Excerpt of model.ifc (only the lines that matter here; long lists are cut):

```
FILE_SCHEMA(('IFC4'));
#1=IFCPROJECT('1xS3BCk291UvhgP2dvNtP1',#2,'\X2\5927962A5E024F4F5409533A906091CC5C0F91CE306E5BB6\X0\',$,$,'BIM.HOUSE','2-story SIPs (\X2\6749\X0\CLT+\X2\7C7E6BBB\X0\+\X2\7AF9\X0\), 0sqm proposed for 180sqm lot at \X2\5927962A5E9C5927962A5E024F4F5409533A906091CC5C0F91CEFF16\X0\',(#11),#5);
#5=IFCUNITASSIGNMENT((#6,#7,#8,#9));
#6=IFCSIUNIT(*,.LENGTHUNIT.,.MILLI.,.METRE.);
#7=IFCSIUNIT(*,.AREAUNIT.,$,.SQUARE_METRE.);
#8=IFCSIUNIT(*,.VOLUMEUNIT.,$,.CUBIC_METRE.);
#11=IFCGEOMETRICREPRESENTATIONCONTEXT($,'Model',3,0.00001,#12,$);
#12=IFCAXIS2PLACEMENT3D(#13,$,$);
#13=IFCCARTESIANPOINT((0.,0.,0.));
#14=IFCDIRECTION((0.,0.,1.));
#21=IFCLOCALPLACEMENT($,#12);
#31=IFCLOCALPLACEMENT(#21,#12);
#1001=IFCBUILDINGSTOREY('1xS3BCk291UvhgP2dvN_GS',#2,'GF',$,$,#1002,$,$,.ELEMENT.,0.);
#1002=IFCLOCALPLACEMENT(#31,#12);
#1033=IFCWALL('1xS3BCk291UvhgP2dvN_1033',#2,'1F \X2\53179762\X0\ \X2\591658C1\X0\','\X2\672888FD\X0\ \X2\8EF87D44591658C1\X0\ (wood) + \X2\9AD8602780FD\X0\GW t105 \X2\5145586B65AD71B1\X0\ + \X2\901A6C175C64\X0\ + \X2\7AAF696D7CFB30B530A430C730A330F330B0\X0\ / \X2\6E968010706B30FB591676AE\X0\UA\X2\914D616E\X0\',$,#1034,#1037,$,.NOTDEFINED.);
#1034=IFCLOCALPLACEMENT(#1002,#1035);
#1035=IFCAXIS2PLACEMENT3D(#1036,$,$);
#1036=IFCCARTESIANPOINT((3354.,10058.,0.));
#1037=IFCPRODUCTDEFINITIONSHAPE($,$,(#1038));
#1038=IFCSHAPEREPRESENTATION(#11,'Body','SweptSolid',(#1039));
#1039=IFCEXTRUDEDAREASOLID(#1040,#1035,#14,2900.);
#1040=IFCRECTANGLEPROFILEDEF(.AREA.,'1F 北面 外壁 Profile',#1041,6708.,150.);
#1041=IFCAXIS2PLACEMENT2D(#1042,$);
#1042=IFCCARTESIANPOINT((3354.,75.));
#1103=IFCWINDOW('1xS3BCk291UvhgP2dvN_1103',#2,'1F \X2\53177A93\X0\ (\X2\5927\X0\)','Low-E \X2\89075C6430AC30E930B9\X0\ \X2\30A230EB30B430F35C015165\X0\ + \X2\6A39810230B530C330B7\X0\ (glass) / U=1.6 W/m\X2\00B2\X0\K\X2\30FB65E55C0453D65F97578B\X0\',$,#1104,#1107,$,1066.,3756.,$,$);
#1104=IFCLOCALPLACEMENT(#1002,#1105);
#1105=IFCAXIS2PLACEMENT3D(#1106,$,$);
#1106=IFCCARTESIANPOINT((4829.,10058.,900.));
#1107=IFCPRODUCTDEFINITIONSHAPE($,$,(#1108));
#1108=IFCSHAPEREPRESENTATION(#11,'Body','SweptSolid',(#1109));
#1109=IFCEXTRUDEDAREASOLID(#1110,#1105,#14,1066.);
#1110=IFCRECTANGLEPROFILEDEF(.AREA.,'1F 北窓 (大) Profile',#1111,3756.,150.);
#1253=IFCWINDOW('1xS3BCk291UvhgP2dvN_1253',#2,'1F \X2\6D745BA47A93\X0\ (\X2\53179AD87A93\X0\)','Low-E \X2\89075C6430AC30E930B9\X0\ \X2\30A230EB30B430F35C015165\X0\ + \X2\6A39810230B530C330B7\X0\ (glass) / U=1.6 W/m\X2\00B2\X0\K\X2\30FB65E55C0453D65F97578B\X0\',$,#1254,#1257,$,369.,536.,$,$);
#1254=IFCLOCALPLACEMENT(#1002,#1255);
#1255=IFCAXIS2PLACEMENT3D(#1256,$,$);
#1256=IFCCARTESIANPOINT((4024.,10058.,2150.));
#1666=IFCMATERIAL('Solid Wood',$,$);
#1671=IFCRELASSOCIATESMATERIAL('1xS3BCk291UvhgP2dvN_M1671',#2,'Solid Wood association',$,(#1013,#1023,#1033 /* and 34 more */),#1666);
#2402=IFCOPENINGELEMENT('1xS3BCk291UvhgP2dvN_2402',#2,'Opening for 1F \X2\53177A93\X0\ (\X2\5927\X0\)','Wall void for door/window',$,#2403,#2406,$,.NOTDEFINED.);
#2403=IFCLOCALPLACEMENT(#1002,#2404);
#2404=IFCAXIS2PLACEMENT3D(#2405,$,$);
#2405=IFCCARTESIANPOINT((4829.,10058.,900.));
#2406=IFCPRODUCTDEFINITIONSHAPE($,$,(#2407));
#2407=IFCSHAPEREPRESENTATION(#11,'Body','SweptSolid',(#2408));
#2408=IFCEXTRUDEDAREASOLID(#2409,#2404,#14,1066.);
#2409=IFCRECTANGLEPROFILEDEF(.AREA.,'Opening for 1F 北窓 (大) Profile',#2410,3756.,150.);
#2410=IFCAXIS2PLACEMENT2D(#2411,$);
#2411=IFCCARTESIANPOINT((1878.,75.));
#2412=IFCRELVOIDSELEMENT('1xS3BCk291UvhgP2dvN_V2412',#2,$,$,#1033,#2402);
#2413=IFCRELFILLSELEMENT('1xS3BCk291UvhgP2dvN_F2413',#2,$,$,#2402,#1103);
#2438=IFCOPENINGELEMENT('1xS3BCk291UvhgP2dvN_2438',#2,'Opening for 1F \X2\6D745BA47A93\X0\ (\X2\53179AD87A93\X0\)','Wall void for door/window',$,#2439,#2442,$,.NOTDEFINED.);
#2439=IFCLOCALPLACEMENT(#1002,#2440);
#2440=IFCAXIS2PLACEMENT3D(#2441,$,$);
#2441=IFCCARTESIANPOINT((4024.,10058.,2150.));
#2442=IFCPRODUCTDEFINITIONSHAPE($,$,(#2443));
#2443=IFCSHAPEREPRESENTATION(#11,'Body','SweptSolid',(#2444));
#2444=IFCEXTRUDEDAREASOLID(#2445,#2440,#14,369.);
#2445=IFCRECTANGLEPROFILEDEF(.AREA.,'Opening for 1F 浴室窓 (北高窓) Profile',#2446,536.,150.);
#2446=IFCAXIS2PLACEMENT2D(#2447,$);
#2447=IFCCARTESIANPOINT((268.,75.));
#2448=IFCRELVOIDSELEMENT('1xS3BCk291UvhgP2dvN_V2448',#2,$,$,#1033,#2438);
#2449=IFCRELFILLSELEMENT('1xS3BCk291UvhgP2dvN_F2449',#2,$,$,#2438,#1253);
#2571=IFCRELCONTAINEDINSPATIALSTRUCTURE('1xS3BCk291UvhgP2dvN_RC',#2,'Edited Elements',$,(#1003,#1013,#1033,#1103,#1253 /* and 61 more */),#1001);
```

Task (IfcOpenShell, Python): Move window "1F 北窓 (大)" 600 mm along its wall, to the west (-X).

```python
import ifcopenshell
import ifcopenshell.api.geometry
import ifcopenshell.util.placement

model = ifcopenshell.open("model.ifc")

window = model.by_id(1103)
opening = window.FillsVoids[0].RelatingOpeningElement
wall = opening.VoidsElements[0].RelatingBuildingElement

wall_matrix = ifcopenshell.util.placement.get_local_placement(wall.ObjectPlacement)
shift = wall_matrix[:3, 0] * -600.0
before = ifcopenshell.util.placement.get_local_placement(window.ObjectPlacement)[:3, 3].copy()

# The window is not placed relative to its opening, so move both.
for product in (opening, window):
    matrix = ifcopenshell.util.placement.get_local_placement(product.ObjectPlacement)
    matrix[:3, 3] += shift
    ifcopenshell.api.geometry.edit_object_placement(model, product=product, matrix=matrix, is_si=False)

after = ifcopenshell.util.placement.get_local_placement(window.ObjectPlacement)[:3, 3]
print("window moved by", (after - before).round(3) + 0.0)

model.write("model_edited.ifc")
```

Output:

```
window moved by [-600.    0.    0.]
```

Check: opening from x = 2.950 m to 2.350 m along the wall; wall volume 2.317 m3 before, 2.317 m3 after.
